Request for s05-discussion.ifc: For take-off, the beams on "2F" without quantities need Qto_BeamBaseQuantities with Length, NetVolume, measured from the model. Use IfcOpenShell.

First a look at what the model holds.

```python
import ifcopenshell
import ifcopenshell.util.element
import ifcopenshell.util.unit

model = ifcopenshell.open("s05-discussion.ifc")
print(model.schema)
for unit_type in ("LENGTHUNIT", "AREAUNIT", "VOLUMEUNIT"):
    print(unit_type, ifcopenshell.util.unit.calculate_unit_scale(model, unit_type))
storey = next(s for s in model.by_type("IfcBuildingStorey") if s.Name == "2F")
beams = [e for e in ifcopenshell.util.element.get_decomposition(storey) if e.is_a("IfcBeam")]
for e in sorted(beams, key=lambda e: e.id()):
    print(e.id(), e.is_a(), e.Name, list(ifcopenshell.util.element.get_psets(e, qtos_only=True)), sep=" | ")
```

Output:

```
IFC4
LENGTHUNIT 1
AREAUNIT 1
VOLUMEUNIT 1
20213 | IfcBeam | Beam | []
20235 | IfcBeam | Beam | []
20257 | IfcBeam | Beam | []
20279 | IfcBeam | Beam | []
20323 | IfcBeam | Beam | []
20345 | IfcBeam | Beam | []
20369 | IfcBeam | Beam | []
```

```python
import ifcopenshell
import ifcopenshell.api.pset
import ifcopenshell.geom
import ifcopenshell.util.element
import ifcopenshell.util.shape
import ifcopenshell.util.unit

model = ifcopenshell.open("s05-discussion.ifc")
unit_scale = ifcopenshell.util.unit.calculate_unit_scale(model)
volume_scale = ifcopenshell.util.unit.calculate_unit_scale(model, "VOLUMEUNIT")
settings = ifcopenshell.geom.settings()

storey = next(s for s in model.by_type("IfcBuildingStorey") if s.Name == "2F")
beams = [e for e in ifcopenshell.util.element.get_decomposition(storey) if e.is_a("IfcBeam")]

for e in sorted(beams, key=lambda e: e.id()):
    if ifcopenshell.util.element.get_psets(e, qtos_only=True, should_inherit=False):
        continue
    # Geometry comes back in metres, in the element's own axes.
    shape = ifcopenshell.geom.create_shape(settings, e)
    values = {
        "Length": ifcopenshell.util.shape.get_max_xyz(shape.geometry) / unit_scale,
        "NetVolume": ifcopenshell.util.shape.get_volume(shape.geometry) / volume_scale,
    }
    qto = ifcopenshell.api.pset.add_qto(model, product=e, name="Qto_BeamBaseQuantities")
    ifcopenshell.api.pset.edit_qto(model, qto=qto, properties=values)
    print(e.id(), {k: round(v, 3) for k, v in values.items()})

model.write("s05-discussion_v2.ifc")
```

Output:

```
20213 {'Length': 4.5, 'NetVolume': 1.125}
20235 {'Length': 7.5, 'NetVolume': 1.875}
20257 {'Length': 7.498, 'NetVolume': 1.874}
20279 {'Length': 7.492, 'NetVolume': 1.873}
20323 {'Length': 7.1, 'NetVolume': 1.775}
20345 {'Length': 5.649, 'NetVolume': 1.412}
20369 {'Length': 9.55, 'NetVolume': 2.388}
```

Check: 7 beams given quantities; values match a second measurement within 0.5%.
